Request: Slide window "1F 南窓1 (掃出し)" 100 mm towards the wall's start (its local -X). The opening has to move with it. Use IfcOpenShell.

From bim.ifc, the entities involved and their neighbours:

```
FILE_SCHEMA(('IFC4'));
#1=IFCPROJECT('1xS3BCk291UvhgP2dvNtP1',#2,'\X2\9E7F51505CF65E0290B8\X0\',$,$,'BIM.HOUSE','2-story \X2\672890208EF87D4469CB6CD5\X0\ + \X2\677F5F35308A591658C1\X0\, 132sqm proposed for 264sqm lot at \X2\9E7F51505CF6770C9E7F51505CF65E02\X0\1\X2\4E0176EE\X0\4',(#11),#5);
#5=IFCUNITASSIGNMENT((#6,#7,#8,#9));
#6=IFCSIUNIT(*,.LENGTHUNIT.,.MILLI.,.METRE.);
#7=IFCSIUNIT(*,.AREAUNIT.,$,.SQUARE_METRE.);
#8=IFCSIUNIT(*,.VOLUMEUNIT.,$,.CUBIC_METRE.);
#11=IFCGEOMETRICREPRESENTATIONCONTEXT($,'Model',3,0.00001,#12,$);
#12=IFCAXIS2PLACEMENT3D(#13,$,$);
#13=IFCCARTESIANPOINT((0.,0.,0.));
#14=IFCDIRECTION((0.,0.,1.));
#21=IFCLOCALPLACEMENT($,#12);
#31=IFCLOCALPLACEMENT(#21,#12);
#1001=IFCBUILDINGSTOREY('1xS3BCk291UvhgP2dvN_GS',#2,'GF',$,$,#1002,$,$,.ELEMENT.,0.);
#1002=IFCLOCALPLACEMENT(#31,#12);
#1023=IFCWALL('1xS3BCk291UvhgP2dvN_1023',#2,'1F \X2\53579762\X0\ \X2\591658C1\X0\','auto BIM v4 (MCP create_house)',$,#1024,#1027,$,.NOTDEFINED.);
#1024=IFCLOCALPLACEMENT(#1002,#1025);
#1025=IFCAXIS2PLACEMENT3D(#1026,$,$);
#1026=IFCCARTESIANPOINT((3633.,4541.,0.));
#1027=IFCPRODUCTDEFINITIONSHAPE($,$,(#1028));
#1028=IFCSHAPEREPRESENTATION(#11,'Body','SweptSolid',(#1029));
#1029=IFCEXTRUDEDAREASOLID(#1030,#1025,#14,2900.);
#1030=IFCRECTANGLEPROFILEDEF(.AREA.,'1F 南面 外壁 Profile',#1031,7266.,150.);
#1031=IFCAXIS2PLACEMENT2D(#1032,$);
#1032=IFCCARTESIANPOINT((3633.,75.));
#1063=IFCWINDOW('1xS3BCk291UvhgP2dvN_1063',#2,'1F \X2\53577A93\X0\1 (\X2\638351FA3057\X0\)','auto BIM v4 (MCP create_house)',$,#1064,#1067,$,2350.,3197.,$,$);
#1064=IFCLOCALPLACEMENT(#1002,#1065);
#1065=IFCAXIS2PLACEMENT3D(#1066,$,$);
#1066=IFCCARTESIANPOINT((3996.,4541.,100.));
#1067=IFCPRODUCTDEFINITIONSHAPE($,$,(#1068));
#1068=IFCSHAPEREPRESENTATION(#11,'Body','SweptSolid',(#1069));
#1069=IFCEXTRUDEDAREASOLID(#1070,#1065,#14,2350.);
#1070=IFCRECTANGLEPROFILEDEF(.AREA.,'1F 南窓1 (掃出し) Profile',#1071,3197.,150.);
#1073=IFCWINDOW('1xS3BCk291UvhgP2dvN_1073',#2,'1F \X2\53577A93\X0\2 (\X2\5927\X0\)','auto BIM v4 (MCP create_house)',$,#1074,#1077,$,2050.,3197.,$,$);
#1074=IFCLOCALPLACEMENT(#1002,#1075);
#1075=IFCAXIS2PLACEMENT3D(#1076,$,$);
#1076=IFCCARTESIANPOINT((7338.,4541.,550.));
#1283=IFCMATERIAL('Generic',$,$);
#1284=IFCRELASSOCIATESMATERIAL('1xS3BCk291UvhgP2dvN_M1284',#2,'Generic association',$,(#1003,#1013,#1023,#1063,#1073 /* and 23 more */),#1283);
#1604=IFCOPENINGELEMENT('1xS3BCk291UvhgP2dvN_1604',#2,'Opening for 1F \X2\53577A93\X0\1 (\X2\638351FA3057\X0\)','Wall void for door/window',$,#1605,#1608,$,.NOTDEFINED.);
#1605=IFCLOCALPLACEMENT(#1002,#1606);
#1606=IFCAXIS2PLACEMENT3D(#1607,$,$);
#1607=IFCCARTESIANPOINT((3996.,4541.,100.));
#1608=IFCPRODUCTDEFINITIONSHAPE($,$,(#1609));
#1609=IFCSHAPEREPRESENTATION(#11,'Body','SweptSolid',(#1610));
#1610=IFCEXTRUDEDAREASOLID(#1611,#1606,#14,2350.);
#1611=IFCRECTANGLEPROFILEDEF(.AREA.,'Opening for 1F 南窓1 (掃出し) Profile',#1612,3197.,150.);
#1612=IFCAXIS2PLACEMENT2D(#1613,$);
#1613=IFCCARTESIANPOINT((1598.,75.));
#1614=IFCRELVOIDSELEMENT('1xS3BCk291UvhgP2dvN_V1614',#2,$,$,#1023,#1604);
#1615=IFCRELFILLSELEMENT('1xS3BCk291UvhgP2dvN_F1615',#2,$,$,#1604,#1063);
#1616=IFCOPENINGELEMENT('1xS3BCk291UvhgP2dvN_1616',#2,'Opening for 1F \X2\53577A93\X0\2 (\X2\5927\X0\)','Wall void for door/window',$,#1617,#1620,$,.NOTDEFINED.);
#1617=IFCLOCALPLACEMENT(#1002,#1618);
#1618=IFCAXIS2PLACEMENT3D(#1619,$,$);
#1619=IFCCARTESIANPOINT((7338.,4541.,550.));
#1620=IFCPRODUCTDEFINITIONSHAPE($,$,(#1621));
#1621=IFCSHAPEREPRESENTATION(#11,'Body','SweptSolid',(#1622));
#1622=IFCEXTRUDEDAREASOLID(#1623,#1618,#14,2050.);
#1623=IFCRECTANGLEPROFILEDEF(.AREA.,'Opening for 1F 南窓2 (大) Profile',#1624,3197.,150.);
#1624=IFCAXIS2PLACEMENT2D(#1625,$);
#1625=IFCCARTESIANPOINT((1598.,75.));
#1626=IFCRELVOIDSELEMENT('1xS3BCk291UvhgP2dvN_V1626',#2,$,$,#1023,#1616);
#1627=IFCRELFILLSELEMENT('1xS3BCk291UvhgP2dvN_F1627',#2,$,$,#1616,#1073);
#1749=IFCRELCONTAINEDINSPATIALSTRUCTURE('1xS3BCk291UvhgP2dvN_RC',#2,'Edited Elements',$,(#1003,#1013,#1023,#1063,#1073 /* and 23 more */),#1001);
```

```python
import ifcopenshell
import ifcopenshell.api.geometry
import ifcopenshell.util.placement
import ifcopenshell.util.unit

model = ifcopenshell.open("bim.ifc")
unit_scale = ifcopenshell.util.unit.calculate_unit_scale(model)

window = model.by_guid("1xS3BCk291UvhgP2dvN_1063")
opening = window.FillsVoids[0].RelatingOpeningElement
wall = opening.VoidsElements[0].RelatingBuildingElement

wall_matrix = ifcopenshell.util.placement.get_local_placement(wall.ObjectPlacement)
shift = wall_matrix[:3, 0] * -0.1 / unit_scale
before = ifcopenshell.util.placement.get_local_placement(window.ObjectPlacement)[:3, 3].copy()

# The window is not placed relative to its opening, so move both.
for product in (opening, window):
    matrix = ifcopenshell.util.placement.get_local_placement(product.ObjectPlacement)
    matrix[:3, 3] += shift
    ifcopenshell.api.geometry.edit_object_placement(model, product=product, matrix=matrix, is_si=False)

after = ifcopenshell.util.placement.get_local_placement(window.ObjectPlacement)[:3, 3]
print("window moved by", (after - before).round(3) + 0.0)

model.write("bim_v2.ifc")
```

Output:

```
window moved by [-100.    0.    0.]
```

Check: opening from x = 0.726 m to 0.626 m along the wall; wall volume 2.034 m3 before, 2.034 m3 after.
